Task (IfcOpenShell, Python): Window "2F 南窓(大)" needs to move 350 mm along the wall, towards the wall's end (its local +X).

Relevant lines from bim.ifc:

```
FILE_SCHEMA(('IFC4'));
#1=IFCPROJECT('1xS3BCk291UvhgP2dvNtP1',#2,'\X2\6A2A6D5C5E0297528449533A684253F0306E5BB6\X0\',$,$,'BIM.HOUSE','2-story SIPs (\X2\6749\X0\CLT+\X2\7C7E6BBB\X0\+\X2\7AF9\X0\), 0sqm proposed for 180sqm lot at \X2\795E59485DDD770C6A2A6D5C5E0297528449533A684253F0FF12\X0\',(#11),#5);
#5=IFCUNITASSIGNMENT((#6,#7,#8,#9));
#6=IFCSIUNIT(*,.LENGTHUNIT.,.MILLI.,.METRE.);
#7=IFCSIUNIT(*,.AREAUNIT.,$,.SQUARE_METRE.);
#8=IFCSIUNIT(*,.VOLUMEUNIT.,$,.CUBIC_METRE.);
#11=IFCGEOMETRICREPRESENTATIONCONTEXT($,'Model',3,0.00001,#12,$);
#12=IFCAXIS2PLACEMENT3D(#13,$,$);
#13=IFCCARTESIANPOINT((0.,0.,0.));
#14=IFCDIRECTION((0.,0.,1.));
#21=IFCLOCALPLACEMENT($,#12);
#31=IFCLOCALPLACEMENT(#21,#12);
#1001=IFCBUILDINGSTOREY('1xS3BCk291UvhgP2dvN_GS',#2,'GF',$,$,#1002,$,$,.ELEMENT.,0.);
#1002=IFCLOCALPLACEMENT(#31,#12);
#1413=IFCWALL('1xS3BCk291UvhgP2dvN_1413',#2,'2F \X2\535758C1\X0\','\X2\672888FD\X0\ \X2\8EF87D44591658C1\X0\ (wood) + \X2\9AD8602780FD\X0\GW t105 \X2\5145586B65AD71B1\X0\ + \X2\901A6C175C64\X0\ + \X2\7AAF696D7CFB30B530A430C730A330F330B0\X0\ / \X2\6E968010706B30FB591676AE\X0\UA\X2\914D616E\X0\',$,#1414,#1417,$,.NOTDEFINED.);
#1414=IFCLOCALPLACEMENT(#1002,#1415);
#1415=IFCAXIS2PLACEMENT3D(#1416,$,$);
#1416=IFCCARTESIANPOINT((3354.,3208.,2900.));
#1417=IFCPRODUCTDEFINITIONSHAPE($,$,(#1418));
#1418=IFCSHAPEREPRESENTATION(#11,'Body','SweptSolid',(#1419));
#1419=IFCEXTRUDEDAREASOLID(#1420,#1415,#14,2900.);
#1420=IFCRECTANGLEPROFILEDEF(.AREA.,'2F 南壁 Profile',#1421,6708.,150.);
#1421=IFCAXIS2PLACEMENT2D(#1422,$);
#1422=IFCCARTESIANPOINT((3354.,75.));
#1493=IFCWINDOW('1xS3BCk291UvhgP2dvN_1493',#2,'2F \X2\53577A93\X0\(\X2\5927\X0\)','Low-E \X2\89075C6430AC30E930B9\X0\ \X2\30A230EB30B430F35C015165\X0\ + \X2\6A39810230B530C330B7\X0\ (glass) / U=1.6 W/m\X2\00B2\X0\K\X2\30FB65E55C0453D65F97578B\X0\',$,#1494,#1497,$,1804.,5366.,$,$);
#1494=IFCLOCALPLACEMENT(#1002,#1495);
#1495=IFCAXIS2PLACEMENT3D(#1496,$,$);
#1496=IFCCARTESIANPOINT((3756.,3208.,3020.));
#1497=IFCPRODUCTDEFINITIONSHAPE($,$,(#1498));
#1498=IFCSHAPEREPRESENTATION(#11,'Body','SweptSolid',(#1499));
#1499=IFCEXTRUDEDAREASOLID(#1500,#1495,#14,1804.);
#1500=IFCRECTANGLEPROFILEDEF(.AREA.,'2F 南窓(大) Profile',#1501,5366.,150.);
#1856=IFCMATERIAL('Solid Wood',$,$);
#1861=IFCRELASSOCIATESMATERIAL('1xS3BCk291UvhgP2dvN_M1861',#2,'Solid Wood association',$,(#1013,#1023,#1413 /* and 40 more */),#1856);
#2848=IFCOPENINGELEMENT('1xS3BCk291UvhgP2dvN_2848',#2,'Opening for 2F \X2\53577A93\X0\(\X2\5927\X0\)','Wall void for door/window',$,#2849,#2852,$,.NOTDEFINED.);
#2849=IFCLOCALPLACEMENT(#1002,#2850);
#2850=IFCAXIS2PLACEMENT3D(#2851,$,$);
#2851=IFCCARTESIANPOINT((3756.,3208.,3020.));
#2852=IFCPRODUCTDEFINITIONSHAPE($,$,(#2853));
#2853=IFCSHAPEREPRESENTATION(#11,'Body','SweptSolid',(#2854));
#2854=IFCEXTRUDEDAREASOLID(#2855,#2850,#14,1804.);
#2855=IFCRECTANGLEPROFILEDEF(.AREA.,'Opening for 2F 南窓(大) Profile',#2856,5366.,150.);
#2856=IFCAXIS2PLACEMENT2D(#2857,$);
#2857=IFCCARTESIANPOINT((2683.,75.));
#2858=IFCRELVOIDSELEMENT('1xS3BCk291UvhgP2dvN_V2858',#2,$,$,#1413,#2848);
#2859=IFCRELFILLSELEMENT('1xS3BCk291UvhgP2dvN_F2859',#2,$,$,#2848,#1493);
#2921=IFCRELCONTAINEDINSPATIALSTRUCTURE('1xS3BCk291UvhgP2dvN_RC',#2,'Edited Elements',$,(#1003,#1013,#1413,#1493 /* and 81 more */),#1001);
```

```python
import ifcopenshell
import ifcopenshell.api.geometry
import ifcopenshell.util.placement
import ifcopenshell.util.unit

model = ifcopenshell.open("bim.ifc")
unit_scale = ifcopenshell.util.unit.calculate_unit_scale(model)

window = model.by_guid("1xS3BCk291UvhgP2dvN_1493")
opening = window.FillsVoids[0].RelatingOpeningElement
wall = opening.VoidsElements[0].RelatingBuildingElement

wall_matrix = ifcopenshell.util.placement.get_local_placement(wall.ObjectPlacement)
shift = wall_matrix[:3, 0] * 0.35 / unit_scale
before = ifcopenshell.util.placement.get_local_placement(window.ObjectPlacement)[:3, 3].copy()

# The window is not placed relative to its opening, so move both.
for product in (opening, window):
    matrix = ifcopenshell.util.placement.get_local_placement(product.ObjectPlacement)
    matrix[:3, 3] += shift
    ifcopenshell.api.geometry.edit_object_placement(model, product=product, matrix=matrix, is_si=False)

after = ifcopenshell.util.placement.get_local_placement(window.ObjectPlacement)[:3, 3]
print("window moved by", (after - before).round(3) + 0.0)

model.write("bim_rev.ifc")
```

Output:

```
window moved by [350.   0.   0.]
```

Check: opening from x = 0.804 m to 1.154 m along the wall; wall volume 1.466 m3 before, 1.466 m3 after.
